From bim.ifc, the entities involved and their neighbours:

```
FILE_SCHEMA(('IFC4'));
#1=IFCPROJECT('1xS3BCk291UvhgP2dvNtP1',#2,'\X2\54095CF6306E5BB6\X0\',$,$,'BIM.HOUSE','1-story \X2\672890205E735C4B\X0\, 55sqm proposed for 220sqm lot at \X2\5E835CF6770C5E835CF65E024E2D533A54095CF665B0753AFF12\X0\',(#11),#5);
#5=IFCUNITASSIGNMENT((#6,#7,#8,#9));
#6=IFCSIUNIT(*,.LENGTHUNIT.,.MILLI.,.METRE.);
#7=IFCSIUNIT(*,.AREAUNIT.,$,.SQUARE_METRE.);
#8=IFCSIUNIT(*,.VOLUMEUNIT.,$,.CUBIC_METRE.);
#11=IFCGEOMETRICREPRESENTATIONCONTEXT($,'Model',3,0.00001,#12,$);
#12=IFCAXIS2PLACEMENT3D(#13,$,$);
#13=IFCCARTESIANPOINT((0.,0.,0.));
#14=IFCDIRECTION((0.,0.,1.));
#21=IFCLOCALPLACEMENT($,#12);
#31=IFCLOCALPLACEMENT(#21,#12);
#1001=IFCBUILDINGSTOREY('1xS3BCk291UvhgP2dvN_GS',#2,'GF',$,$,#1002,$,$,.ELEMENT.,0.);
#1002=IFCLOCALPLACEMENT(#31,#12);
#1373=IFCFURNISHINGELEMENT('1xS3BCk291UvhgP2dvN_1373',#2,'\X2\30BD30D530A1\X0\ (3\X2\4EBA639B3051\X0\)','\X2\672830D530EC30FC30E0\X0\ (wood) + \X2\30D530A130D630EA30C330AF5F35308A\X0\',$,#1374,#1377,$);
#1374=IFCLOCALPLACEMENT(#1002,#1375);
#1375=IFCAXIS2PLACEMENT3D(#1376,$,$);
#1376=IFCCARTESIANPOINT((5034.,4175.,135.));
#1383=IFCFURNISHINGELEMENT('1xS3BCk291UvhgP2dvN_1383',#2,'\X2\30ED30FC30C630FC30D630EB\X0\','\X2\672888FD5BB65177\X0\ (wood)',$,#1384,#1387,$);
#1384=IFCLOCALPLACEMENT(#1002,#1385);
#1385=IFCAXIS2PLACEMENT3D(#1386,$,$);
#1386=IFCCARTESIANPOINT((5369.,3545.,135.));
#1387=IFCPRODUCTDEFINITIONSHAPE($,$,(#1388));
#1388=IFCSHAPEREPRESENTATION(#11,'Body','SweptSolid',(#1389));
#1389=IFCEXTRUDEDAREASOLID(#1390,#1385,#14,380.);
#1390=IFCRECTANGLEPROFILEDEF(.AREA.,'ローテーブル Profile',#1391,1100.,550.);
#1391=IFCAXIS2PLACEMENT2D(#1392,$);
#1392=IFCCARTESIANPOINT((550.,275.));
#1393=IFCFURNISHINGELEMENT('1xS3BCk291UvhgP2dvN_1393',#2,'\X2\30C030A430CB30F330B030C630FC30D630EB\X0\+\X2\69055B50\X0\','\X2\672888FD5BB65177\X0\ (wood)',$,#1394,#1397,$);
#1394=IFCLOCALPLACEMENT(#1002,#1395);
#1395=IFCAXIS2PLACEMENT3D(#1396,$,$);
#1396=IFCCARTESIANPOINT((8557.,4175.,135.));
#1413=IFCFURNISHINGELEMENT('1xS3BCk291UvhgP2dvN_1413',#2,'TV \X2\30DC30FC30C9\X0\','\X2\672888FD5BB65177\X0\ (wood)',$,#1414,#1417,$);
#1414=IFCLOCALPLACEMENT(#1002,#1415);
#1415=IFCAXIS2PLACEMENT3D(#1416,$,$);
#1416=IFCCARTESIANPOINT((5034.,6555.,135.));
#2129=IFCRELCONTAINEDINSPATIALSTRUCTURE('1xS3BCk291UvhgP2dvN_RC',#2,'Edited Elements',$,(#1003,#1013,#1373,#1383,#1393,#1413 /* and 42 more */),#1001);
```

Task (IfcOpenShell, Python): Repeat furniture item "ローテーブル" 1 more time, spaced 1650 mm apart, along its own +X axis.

```python
import ifcopenshell
import ifcopenshell.api.geometry
import ifcopenshell.api.root
import ifcopenshell.util.element
import ifcopenshell.util.placement

model = ifcopenshell.open("bim.ifc")


def reuse_history(source, copy):
    """copy_class also copies each property set's owner history, people and application; keep the originals."""
    for rel in copy.IsDefinedBy:
        if rel.is_a("IfcRelDefinesByProperties") and (history := rel.RelatingPropertyDefinition.OwnerHistory):
            rel.RelatingPropertyDefinition.OwnerHistory = source.OwnerHistory
            ifcopenshell.util.element.remove_deep2(model, history)


source = model.by_guid("1xS3BCk291UvhgP2dvN_1383")
base = ifcopenshell.util.placement.get_local_placement(source.ObjectPlacement)
step = base[:3, 0] * 1650.0

for i in range(1, 2):
    copy = ifcopenshell.api.root.copy_class(model, product=source)
    copy.Representation = ifcopenshell.util.element.copy_deep(
        model, source.Representation, exclude=["IfcGeometricRepresentationContext", "IfcRepresentationMap"]
    )
    reuse_history(source, copy)
    matrix = base.copy()
    matrix[:3, 3] += i * step
    print("added at", matrix[:3, 3].round(3) + 0.0)
    ifcopenshell.api.geometry.edit_object_placement(model, product=copy, matrix=matrix, is_si=False)

model.write("bim-out.ifc")
```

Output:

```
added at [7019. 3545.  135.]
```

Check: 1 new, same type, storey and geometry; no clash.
